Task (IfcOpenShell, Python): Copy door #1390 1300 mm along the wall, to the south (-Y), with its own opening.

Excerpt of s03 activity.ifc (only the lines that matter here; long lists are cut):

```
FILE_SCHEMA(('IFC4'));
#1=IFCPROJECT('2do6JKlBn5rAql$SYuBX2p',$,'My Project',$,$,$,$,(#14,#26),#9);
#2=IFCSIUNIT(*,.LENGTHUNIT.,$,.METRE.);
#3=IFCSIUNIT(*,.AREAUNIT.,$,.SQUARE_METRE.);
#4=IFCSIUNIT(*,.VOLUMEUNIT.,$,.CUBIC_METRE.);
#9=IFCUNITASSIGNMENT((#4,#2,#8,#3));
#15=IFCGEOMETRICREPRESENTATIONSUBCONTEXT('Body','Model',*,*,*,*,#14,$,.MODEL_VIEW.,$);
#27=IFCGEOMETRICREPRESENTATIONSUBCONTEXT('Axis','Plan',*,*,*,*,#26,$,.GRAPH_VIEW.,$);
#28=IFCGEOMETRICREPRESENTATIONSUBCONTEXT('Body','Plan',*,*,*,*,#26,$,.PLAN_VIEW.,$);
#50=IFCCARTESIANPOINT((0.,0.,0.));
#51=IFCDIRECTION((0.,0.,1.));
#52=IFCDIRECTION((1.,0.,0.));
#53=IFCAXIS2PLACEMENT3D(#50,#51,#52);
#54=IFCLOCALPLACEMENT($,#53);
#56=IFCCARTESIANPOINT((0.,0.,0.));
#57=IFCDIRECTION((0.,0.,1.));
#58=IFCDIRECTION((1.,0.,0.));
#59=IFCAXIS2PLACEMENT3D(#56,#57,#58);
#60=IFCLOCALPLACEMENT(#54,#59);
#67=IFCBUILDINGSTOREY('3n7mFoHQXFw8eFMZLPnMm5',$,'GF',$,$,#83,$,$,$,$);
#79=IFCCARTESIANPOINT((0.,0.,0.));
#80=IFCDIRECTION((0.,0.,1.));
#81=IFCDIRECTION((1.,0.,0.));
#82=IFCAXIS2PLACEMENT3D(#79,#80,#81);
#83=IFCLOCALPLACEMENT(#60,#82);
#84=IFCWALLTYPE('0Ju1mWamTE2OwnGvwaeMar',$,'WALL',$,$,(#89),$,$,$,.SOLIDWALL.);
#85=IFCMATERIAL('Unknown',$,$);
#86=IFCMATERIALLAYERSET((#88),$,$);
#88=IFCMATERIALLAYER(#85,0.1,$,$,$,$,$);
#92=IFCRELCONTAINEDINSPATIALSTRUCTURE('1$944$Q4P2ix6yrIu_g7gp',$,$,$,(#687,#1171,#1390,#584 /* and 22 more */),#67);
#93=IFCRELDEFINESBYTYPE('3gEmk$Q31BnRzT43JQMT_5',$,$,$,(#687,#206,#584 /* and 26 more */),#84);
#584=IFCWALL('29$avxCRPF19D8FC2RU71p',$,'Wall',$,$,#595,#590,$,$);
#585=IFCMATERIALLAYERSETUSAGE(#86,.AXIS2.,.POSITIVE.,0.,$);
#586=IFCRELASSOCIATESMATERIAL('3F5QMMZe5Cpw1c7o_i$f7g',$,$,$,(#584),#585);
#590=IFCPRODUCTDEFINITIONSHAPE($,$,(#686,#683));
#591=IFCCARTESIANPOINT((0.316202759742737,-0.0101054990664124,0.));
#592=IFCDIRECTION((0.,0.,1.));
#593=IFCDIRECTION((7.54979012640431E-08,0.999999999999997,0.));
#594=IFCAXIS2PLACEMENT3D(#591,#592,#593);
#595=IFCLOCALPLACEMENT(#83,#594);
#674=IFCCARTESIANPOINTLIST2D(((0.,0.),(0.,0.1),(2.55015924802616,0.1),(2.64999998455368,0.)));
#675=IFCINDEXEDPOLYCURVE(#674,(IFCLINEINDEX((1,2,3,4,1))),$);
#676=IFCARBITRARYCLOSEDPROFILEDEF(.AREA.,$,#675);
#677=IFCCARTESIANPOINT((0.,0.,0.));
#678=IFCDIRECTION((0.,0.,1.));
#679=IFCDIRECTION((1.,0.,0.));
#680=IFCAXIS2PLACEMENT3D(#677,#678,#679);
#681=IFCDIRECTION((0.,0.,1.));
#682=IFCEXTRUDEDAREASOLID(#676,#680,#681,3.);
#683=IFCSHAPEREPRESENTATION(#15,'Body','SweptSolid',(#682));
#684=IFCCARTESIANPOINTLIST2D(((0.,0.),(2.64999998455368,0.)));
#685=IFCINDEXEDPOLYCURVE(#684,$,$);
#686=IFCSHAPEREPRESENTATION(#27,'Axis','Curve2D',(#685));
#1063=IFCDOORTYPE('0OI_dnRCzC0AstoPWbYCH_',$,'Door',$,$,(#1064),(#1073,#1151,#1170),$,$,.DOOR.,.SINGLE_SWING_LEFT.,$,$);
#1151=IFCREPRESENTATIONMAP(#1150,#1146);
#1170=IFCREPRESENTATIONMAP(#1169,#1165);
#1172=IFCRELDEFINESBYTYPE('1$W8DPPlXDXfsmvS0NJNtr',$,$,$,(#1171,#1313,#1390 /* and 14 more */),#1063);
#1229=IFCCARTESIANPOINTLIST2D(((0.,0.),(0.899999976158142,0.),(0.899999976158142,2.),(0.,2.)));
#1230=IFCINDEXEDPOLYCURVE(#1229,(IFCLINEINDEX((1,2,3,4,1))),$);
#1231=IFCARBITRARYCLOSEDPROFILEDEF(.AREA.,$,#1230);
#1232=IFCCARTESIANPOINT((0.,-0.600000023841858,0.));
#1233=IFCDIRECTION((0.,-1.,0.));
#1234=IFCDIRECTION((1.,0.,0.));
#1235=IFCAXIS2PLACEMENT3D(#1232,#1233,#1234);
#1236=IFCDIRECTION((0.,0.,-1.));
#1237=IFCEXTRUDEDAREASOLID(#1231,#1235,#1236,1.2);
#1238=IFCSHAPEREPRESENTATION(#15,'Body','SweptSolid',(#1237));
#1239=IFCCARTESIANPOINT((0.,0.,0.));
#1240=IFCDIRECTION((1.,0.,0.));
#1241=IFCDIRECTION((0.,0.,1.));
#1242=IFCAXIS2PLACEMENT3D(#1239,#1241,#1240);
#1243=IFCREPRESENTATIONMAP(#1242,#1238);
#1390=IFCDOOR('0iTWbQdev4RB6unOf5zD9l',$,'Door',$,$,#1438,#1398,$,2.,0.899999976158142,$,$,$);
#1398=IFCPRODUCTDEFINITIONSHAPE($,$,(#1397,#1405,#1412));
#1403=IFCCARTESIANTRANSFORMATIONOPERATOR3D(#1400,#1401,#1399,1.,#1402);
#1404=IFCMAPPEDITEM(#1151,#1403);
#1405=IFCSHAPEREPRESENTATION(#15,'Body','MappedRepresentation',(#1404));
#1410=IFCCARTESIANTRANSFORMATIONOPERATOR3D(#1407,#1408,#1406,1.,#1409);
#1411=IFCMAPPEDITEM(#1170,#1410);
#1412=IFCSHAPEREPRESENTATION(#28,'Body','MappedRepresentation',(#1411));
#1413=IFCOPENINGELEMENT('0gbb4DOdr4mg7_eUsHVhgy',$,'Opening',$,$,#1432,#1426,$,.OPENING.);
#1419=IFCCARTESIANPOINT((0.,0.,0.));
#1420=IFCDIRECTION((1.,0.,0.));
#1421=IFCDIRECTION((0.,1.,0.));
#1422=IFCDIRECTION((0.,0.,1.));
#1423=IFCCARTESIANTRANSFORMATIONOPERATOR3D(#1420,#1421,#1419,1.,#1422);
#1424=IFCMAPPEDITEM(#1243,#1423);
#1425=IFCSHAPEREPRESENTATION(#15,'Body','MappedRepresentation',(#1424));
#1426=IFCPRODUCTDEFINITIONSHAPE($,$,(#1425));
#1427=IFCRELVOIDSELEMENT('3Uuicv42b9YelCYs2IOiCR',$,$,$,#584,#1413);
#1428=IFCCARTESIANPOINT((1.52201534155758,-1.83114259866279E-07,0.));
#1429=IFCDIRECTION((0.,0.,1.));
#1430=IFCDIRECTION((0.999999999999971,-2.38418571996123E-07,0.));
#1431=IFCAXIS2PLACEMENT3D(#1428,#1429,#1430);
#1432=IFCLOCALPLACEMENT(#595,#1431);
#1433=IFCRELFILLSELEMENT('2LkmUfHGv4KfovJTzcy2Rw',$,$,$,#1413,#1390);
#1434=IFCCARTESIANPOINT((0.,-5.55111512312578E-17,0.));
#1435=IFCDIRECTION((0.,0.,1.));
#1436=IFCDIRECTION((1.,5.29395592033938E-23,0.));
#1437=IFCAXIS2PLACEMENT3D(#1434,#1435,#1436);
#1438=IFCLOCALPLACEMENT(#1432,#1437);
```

```python
import ifcopenshell
import ifcopenshell.api.feature
import ifcopenshell.api.geometry
import ifcopenshell.api.root
import ifcopenshell.geom
import ifcopenshell.util.element
import ifcopenshell.util.placement
import ifcopenshell.util.shape
import ifcopenshell.util.unit

model = ifcopenshell.open("s03 activity.ifc")
unit_scale = ifcopenshell.util.unit.calculate_unit_scale(model)
settings = ifcopenshell.geom.settings()


def volume(element):
    """Net volume in cubic metres, openings subtracted."""
    shape = ifcopenshell.geom.create_shape(settings, element)
    return ifcopenshell.util.shape.get_volume(shape.geometry)


door = model.by_id(1390)
opening = door.FillsVoids[0].RelatingOpeningElement
wall = opening.VoidsElements[0].RelatingBuildingElement
before = volume(wall)
shift = ifcopenshell.util.placement.get_local_placement(wall.ObjectPlacement)[:3, 0] * -1.3 / unit_scale

# copy_class copies the void relationship, type, container and properties, but no geometry.
new_opening = ifcopenshell.api.root.copy_class(model, product=opening)
new_opening.Representation = ifcopenshell.util.element.copy_deep(
    model, opening.Representation, exclude=["IfcGeometricRepresentationContext", "IfcRepresentationMap"]
)
new_door = ifcopenshell.api.root.copy_class(model, product=door)
new_door.Representation = ifcopenshell.util.element.copy_deep(
    model, door.Representation, exclude=["IfcGeometricRepresentationContext", "IfcRepresentationMap"]
)
ifcopenshell.api.feature.add_filling(model, opening=new_opening, element=new_door)

for old, new in ((opening, new_opening), (door, new_door)):
    matrix = ifcopenshell.util.placement.get_local_placement(old.ObjectPlacement)
    matrix[:3, 3] += shift
    ifcopenshell.api.geometry.edit_object_placement(model, product=new, matrix=matrix, is_si=False)

after = volume(wall)

print(f"wall volume {before:.3f} -> {after:.3f} m3")

model.write("s03 activity_rev.ifc")
```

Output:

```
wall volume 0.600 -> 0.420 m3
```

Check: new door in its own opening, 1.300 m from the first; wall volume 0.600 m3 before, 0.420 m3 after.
